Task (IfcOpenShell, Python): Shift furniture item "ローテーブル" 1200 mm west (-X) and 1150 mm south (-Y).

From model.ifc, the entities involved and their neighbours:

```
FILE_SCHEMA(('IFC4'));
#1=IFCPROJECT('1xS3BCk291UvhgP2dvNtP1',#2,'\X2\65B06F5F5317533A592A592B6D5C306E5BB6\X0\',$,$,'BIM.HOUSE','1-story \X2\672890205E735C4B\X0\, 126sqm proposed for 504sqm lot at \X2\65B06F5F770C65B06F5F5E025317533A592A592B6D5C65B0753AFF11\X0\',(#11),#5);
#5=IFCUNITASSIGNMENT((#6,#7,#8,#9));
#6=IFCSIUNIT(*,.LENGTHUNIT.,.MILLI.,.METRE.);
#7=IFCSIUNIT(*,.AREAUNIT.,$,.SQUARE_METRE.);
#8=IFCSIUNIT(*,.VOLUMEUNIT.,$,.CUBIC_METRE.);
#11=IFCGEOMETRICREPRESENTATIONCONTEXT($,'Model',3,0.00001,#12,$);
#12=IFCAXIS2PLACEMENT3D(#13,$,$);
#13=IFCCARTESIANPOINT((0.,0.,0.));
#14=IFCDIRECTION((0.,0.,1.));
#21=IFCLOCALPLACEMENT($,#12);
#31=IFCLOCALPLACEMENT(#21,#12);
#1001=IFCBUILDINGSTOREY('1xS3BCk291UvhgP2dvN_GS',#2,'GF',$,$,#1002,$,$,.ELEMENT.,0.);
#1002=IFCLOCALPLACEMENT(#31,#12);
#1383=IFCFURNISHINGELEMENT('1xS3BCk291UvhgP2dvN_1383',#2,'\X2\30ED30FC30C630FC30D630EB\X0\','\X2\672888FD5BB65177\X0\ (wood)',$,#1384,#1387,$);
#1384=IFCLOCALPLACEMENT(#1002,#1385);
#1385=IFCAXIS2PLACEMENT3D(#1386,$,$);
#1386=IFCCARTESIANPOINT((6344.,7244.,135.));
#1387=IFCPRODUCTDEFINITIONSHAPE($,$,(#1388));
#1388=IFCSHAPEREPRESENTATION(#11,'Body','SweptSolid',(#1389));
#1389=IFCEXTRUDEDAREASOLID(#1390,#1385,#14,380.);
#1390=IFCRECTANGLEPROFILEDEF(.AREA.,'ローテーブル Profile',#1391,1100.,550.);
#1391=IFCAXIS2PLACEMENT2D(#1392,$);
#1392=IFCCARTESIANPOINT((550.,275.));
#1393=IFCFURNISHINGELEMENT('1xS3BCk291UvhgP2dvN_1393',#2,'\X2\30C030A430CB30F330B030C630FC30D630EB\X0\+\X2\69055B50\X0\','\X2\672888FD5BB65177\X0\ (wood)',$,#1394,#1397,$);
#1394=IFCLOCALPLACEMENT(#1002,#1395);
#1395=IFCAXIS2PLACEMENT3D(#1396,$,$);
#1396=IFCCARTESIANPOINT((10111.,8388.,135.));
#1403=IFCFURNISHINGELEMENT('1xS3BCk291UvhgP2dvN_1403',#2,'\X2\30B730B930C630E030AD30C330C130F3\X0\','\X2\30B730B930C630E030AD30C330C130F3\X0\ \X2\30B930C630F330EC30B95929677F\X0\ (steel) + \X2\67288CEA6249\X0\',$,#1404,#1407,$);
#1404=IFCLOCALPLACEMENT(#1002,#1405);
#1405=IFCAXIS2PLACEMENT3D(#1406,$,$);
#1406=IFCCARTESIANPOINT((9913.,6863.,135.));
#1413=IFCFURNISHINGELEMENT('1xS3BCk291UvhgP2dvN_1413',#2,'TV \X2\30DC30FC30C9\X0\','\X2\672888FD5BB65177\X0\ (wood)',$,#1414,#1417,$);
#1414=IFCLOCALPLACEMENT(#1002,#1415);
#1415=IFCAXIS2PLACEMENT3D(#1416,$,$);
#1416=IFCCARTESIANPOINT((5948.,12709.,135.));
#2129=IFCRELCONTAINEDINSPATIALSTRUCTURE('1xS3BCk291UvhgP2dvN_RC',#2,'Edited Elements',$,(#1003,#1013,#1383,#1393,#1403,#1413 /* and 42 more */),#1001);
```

```python
import ifcopenshell
import ifcopenshell.api.geometry
import ifcopenshell.util.placement
import ifcopenshell.util.unit

model = ifcopenshell.open("model.ifc")
unit_scale = ifcopenshell.util.unit.calculate_unit_scale(model)

item = model.by_guid("1xS3BCk291UvhgP2dvN_1383")
matrix = ifcopenshell.util.placement.get_local_placement(item.ObjectPlacement)
matrix[0, 3] -= 1.2 / unit_scale
matrix[1, 3] -= 1.15 / unit_scale
ifcopenshell.api.geometry.edit_object_placement(model, product=item, matrix=matrix, is_si=False)

print(ifcopenshell.util.placement.get_local_placement(item.ObjectPlacement).round(3) + 0.0)

model.write("model-out.ifc")
```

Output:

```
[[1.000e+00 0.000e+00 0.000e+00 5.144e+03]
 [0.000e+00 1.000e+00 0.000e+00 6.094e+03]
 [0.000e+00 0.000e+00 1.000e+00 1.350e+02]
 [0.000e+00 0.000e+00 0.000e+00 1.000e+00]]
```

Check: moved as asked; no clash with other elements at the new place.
